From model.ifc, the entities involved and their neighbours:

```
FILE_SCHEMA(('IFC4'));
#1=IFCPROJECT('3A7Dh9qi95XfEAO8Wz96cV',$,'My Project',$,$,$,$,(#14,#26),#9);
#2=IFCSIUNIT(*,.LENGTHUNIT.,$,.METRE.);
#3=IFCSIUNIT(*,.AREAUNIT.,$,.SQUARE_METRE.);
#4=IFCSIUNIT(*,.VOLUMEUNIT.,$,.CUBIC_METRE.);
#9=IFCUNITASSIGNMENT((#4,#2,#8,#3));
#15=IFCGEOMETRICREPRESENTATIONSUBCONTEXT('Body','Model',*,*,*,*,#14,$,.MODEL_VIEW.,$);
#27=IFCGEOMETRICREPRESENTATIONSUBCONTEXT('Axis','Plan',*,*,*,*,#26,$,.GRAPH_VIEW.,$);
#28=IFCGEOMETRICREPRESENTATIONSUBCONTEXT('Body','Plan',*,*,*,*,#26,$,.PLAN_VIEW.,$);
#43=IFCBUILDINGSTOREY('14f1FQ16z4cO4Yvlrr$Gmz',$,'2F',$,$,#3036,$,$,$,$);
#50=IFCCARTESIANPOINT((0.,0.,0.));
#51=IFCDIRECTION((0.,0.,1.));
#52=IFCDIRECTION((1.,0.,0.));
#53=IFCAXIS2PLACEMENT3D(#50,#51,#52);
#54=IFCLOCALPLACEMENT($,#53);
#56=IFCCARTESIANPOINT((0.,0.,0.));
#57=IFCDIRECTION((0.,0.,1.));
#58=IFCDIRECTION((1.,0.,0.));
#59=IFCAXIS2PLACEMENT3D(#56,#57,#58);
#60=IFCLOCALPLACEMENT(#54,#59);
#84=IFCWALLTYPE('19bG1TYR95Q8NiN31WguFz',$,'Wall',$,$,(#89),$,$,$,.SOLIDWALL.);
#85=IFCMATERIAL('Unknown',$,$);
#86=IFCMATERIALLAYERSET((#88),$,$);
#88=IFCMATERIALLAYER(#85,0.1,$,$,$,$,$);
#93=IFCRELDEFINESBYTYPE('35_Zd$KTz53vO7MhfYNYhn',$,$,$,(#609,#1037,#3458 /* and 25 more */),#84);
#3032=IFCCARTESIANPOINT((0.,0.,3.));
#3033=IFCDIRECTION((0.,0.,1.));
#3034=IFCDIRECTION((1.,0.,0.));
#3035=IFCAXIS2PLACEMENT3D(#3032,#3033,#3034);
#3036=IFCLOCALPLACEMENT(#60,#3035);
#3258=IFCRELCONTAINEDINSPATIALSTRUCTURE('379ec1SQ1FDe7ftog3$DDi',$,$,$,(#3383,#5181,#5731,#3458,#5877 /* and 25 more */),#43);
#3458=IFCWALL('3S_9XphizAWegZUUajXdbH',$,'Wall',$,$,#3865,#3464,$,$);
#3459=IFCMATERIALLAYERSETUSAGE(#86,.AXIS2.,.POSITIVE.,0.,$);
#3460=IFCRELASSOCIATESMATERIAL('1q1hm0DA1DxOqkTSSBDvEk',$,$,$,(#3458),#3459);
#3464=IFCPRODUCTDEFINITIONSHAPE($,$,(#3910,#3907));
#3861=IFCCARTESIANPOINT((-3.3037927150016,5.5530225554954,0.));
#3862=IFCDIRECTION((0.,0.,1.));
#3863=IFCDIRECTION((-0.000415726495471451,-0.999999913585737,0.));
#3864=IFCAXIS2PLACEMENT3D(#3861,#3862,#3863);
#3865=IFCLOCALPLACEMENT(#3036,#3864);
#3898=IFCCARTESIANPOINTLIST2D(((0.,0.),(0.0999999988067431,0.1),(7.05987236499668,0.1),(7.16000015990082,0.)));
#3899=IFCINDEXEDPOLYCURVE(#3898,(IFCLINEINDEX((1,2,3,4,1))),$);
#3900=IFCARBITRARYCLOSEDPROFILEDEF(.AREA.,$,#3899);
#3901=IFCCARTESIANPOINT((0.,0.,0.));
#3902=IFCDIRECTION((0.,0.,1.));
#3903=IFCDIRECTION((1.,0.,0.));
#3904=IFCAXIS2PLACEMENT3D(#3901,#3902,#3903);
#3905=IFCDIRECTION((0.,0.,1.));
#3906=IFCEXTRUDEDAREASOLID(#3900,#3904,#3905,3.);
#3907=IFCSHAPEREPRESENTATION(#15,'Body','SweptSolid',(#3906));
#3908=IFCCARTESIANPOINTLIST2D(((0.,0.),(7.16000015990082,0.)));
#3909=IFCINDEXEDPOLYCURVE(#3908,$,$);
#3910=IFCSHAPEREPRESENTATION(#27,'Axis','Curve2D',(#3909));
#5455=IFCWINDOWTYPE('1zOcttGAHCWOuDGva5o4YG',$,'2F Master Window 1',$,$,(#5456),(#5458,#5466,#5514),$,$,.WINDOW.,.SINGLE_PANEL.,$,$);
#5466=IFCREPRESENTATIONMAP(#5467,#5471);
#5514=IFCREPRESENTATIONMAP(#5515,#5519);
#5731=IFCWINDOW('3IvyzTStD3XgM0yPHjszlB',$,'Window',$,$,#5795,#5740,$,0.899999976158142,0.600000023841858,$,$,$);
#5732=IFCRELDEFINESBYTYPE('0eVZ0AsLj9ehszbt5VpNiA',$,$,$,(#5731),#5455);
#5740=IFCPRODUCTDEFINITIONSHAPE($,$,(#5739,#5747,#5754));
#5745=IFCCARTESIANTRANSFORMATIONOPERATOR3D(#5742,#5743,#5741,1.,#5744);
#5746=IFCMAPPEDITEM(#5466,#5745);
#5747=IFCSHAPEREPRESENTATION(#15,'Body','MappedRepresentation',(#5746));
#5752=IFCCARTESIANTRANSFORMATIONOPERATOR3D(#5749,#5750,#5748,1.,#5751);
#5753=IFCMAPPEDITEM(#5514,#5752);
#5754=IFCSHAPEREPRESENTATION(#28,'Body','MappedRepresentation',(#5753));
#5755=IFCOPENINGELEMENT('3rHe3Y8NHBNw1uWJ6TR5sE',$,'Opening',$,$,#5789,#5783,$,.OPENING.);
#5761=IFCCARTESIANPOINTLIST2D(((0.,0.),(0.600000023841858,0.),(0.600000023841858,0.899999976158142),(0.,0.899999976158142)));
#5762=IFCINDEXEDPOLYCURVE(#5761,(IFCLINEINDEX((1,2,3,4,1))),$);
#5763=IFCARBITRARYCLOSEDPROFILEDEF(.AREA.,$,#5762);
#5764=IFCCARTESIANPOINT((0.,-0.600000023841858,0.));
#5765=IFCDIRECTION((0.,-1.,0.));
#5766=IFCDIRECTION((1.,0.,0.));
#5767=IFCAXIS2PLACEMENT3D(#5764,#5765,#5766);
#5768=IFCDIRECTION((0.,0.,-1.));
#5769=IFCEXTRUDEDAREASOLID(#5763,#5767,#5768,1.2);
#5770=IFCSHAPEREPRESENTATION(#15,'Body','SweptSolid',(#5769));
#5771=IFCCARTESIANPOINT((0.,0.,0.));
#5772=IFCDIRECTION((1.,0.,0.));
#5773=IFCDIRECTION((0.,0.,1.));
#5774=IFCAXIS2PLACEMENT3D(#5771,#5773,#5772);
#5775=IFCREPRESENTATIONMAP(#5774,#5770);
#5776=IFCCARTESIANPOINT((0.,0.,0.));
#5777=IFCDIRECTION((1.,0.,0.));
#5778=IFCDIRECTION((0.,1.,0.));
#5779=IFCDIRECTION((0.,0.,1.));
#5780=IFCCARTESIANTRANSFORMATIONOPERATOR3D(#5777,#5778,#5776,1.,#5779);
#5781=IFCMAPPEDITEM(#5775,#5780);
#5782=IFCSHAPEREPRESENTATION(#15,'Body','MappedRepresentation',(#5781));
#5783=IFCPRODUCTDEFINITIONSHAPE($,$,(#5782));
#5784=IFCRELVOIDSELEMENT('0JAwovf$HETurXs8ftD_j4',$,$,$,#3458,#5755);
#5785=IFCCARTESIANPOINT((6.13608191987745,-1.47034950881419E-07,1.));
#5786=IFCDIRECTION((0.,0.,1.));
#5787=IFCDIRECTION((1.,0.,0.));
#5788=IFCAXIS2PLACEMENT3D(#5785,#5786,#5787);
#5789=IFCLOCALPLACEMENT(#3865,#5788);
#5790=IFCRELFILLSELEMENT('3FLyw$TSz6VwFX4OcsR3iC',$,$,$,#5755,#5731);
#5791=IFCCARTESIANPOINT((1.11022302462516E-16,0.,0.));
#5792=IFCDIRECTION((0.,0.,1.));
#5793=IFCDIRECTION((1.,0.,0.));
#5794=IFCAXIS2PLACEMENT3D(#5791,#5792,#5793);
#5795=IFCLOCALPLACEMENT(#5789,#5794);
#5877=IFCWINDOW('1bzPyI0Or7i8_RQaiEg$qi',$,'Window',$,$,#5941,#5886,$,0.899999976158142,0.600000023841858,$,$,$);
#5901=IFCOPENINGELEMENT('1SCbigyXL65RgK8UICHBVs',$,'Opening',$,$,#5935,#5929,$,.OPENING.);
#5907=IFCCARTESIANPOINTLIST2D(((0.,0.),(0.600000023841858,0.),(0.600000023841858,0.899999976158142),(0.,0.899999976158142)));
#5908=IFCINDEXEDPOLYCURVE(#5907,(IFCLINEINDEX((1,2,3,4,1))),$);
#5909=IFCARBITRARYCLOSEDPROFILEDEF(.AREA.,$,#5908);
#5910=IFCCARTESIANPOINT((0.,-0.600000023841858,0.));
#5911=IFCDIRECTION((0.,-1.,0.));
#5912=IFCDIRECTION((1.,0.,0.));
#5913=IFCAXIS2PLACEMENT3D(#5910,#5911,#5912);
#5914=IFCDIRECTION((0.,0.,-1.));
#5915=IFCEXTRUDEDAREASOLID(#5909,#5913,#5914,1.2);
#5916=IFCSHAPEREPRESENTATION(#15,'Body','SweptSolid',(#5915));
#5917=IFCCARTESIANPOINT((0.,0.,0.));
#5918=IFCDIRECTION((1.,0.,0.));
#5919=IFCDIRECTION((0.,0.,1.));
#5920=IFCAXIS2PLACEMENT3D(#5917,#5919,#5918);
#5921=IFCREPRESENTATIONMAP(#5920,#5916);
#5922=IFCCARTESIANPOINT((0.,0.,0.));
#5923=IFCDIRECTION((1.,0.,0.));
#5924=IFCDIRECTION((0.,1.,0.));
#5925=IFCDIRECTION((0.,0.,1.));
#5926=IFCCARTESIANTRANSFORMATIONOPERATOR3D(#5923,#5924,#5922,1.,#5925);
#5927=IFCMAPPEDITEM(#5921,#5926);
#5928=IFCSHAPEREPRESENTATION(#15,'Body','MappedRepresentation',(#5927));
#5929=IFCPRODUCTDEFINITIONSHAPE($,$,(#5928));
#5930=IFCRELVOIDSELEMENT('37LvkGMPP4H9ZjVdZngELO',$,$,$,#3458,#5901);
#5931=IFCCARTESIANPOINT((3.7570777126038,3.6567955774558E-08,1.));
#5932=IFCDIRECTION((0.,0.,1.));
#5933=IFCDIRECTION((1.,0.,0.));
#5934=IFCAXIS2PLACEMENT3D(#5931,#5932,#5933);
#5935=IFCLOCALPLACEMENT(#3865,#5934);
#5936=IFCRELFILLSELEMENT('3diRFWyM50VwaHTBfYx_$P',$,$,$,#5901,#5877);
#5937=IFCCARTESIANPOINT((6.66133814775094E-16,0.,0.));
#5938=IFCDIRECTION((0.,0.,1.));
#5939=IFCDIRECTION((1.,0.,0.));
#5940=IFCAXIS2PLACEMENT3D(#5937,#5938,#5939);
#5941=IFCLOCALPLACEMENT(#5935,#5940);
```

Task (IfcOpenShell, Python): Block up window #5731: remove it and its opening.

```python
import ifcopenshell
import ifcopenshell.api.feature
import ifcopenshell.api.root
import ifcopenshell.geom
import ifcopenshell.util.shape

model = ifcopenshell.open("model.ifc")
settings = ifcopenshell.geom.settings()


def volume(element):
    """Net volume in cubic metres, openings subtracted."""
    shape = ifcopenshell.geom.create_shape(settings, element)
    return ifcopenshell.util.shape.get_volume(shape.geometry)


window = model.by_guid("3IvyzTStD3XgM0yPHjszlB")
opening = window.FillsVoids[0].RelatingOpeningElement
wall = opening.VoidsElements[0].RelatingBuildingElement
before = volume(wall)

ifcopenshell.api.root.remove_product(model, product=window)
ifcopenshell.api.feature.remove_feature(model, feature=opening)

after = volume(wall)

print(f"wall volume {before:.3f} -> {after:.3f} m3")

model.write("model_rev.ifc")
```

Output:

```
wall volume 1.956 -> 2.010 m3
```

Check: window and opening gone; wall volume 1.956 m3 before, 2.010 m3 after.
